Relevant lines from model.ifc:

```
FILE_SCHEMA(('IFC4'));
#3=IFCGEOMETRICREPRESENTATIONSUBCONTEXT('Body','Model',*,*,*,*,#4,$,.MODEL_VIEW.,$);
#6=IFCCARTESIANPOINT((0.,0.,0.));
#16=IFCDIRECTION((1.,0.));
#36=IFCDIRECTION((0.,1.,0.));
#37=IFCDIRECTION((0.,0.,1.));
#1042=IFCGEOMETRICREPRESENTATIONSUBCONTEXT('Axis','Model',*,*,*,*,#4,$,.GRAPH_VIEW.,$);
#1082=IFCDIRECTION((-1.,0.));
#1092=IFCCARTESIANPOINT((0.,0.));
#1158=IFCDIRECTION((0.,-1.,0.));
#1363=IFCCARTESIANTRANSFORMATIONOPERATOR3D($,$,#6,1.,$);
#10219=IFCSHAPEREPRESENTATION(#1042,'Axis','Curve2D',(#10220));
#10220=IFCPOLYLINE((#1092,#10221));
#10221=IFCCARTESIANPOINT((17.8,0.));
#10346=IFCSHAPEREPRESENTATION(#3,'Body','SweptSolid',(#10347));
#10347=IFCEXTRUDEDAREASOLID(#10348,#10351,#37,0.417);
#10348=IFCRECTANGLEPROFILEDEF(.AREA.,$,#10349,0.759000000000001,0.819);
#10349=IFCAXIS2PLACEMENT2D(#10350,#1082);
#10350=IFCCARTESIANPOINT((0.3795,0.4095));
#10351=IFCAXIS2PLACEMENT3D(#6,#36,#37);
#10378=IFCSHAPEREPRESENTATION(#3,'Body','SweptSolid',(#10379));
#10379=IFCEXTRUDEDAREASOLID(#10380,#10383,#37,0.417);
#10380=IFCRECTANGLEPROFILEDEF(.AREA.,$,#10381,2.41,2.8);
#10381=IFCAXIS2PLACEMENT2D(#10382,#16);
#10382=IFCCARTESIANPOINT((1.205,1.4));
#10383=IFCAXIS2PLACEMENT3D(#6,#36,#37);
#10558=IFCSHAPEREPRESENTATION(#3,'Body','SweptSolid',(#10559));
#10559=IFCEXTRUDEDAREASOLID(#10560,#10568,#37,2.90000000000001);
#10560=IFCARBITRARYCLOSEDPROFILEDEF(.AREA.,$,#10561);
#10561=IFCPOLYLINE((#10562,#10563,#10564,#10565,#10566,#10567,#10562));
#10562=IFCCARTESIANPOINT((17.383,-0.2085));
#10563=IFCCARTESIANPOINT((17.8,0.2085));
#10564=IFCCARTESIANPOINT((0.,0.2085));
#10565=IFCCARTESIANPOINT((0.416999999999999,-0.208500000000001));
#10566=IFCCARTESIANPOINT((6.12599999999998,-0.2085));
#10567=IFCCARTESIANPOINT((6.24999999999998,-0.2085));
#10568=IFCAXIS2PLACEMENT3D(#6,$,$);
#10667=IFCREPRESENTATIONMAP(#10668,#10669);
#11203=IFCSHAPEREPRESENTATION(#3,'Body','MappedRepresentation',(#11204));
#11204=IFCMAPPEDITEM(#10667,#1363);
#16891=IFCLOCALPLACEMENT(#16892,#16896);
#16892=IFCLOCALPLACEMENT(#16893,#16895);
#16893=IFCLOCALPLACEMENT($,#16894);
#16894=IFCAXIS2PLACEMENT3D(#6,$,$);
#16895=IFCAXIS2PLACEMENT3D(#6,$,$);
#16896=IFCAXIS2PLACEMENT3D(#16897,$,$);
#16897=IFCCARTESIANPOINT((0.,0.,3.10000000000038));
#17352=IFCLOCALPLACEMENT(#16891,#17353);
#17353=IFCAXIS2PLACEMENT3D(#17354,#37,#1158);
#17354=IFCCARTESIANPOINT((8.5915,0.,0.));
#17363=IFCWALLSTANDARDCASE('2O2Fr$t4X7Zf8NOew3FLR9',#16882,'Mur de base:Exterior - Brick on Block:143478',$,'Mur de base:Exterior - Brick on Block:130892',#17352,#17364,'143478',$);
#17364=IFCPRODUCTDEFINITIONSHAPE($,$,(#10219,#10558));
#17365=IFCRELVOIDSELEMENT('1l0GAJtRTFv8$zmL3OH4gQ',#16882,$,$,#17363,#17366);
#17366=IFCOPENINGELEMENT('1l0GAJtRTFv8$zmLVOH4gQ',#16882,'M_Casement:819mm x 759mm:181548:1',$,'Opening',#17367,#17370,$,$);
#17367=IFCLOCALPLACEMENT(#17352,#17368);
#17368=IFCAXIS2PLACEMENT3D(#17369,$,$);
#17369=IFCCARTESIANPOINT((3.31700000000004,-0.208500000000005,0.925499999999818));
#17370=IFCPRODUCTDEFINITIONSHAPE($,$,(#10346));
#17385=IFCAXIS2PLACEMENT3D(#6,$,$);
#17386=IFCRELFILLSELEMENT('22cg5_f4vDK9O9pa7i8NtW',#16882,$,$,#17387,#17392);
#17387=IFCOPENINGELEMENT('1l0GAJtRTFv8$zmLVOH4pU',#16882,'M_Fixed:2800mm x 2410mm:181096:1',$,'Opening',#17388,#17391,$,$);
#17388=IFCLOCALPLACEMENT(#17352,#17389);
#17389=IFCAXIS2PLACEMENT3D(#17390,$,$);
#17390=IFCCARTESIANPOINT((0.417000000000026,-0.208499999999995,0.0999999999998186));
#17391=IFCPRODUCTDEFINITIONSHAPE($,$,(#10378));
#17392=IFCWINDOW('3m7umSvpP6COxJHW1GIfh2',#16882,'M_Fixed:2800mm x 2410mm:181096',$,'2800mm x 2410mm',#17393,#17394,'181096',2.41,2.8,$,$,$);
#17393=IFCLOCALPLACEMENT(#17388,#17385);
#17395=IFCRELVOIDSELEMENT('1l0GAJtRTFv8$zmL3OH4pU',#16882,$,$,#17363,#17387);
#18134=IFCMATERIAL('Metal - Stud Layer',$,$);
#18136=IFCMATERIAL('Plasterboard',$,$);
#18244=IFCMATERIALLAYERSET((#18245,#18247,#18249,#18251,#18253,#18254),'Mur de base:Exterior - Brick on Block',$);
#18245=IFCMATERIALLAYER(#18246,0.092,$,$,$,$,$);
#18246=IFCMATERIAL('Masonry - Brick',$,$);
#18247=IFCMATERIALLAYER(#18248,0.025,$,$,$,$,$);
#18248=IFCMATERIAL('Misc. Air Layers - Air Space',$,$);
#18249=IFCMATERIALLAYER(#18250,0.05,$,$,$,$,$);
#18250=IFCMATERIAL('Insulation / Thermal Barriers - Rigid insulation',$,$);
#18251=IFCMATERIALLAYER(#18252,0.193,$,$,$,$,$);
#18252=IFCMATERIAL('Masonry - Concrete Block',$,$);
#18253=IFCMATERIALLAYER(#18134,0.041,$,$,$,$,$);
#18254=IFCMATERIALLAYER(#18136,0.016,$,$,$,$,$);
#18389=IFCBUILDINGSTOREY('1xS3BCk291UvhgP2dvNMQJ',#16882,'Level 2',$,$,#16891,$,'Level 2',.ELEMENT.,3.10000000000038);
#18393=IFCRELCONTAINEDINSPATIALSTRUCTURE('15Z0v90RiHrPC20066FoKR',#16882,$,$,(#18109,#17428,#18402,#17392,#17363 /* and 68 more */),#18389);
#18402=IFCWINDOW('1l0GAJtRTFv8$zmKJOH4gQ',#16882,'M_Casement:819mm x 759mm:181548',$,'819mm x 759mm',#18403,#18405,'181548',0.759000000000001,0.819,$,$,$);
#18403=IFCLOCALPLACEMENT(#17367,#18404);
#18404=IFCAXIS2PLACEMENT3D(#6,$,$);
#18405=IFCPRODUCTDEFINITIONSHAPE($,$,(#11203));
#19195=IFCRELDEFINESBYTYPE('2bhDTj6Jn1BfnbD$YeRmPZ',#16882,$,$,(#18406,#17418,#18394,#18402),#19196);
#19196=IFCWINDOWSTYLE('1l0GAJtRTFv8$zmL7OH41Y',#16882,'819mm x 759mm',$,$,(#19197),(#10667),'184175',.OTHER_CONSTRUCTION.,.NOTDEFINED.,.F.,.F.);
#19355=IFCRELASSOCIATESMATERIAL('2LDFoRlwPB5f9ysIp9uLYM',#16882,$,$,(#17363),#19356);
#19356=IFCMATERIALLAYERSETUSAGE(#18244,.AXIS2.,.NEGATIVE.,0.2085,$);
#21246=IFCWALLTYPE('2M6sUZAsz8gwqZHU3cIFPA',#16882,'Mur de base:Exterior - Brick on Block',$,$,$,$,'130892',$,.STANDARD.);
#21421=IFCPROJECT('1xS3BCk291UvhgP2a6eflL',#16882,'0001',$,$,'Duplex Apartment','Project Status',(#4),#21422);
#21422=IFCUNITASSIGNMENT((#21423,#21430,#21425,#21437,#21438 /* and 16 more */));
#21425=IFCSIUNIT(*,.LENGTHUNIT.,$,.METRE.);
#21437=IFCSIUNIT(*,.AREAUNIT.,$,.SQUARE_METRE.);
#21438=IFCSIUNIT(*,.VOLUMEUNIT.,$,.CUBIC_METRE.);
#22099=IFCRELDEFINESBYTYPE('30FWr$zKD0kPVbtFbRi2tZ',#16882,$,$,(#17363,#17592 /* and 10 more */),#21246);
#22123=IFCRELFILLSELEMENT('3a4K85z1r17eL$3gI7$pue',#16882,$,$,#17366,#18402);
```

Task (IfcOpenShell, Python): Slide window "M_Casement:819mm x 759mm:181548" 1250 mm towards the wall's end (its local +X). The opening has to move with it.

```python
import ifcopenshell
import ifcopenshell.api.geometry
import ifcopenshell.util.placement

model = ifcopenshell.open("model.ifc")

window = model.by_guid("1l0GAJtRTFv8$zmKJOH4gQ")
opening = window.FillsVoids[0].RelatingOpeningElement
wall = opening.VoidsElements[0].RelatingBuildingElement

wall_matrix = ifcopenshell.util.placement.get_local_placement(wall.ObjectPlacement)
shift = wall_matrix[:3, 0] * 1.25
before = ifcopenshell.util.placement.get_local_placement(window.ObjectPlacement)[:3, 3].copy()

# The window is placed relative to its opening, so it follows when the opening moves.
matrix = ifcopenshell.util.placement.get_local_placement(opening.ObjectPlacement)
matrix[:3, 3] += shift
ifcopenshell.api.geometry.edit_object_placement(
    model, product=opening, matrix=matrix, is_si=False, should_transform_children=True
)

after = ifcopenshell.util.placement.get_local_placement(window.ObjectPlacement)[:3, 3]
print("window moved by", (after - before).round(3) + 0.0)

model.write("model-out.ifc")
```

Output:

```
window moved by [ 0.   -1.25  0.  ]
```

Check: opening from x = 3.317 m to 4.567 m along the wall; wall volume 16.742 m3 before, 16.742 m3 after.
